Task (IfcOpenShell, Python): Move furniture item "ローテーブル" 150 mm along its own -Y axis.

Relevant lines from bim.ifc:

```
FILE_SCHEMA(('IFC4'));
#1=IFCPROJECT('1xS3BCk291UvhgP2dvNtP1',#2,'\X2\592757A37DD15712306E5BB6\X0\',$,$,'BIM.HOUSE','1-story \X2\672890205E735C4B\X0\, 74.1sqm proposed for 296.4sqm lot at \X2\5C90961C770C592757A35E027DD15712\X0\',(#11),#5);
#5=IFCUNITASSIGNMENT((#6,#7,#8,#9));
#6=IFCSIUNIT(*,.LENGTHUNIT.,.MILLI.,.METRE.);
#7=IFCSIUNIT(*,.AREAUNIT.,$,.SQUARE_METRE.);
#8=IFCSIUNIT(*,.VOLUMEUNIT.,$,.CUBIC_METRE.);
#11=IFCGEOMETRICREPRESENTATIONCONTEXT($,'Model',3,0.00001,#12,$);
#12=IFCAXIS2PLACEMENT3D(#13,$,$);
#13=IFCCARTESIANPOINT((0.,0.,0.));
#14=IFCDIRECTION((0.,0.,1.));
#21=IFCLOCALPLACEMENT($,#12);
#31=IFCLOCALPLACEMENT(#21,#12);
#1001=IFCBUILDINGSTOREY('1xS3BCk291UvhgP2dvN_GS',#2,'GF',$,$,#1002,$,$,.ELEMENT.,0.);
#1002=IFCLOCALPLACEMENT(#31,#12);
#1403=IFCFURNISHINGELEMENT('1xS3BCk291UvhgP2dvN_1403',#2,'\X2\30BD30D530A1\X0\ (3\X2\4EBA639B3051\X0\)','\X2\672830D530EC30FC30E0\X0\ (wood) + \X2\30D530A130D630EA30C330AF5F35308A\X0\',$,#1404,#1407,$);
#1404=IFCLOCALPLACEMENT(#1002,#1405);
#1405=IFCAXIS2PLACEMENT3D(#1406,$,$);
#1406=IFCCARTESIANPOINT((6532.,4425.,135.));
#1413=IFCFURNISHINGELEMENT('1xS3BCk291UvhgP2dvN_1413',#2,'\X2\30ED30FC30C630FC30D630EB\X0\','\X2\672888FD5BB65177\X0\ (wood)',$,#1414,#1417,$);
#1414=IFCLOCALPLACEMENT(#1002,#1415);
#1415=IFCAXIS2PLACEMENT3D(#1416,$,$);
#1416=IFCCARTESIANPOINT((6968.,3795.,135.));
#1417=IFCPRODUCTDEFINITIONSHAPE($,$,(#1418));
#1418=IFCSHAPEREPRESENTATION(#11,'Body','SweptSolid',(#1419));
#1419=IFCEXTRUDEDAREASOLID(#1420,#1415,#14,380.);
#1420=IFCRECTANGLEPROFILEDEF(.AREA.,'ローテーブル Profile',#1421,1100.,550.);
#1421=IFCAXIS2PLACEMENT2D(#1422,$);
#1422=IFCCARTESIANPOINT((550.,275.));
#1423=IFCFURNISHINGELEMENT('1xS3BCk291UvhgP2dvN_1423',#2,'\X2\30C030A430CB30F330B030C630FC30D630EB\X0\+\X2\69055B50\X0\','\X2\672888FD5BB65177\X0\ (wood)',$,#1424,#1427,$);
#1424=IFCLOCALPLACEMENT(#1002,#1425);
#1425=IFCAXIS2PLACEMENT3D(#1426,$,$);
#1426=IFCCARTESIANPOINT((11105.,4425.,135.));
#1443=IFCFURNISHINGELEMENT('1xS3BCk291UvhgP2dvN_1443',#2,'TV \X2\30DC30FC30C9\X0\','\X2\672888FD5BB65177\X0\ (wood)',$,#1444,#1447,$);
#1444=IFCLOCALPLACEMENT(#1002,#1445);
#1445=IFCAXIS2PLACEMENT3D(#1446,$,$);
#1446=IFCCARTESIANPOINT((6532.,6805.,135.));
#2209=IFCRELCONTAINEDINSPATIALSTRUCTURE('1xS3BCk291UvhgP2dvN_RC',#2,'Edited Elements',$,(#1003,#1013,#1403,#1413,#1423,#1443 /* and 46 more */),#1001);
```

```python
import ifcopenshell
import ifcopenshell.api.geometry
import ifcopenshell.util.placement

model = ifcopenshell.open("bim.ifc")

item = model.by_id(1413)
matrix = ifcopenshell.util.placement.get_local_placement(item.ObjectPlacement)
matrix[:3, 3] -= matrix[:3, 1] * 150.0
ifcopenshell.api.geometry.edit_object_placement(model, product=item, matrix=matrix, is_si=False)

print(ifcopenshell.util.placement.get_local_placement(item.ObjectPlacement).round(3) + 0.0)

model.write("bim_v2.ifc")
```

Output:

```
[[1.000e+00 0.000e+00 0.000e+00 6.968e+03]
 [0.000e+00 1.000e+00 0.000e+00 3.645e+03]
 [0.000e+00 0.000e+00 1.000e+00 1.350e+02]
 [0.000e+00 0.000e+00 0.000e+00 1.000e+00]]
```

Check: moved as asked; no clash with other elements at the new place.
